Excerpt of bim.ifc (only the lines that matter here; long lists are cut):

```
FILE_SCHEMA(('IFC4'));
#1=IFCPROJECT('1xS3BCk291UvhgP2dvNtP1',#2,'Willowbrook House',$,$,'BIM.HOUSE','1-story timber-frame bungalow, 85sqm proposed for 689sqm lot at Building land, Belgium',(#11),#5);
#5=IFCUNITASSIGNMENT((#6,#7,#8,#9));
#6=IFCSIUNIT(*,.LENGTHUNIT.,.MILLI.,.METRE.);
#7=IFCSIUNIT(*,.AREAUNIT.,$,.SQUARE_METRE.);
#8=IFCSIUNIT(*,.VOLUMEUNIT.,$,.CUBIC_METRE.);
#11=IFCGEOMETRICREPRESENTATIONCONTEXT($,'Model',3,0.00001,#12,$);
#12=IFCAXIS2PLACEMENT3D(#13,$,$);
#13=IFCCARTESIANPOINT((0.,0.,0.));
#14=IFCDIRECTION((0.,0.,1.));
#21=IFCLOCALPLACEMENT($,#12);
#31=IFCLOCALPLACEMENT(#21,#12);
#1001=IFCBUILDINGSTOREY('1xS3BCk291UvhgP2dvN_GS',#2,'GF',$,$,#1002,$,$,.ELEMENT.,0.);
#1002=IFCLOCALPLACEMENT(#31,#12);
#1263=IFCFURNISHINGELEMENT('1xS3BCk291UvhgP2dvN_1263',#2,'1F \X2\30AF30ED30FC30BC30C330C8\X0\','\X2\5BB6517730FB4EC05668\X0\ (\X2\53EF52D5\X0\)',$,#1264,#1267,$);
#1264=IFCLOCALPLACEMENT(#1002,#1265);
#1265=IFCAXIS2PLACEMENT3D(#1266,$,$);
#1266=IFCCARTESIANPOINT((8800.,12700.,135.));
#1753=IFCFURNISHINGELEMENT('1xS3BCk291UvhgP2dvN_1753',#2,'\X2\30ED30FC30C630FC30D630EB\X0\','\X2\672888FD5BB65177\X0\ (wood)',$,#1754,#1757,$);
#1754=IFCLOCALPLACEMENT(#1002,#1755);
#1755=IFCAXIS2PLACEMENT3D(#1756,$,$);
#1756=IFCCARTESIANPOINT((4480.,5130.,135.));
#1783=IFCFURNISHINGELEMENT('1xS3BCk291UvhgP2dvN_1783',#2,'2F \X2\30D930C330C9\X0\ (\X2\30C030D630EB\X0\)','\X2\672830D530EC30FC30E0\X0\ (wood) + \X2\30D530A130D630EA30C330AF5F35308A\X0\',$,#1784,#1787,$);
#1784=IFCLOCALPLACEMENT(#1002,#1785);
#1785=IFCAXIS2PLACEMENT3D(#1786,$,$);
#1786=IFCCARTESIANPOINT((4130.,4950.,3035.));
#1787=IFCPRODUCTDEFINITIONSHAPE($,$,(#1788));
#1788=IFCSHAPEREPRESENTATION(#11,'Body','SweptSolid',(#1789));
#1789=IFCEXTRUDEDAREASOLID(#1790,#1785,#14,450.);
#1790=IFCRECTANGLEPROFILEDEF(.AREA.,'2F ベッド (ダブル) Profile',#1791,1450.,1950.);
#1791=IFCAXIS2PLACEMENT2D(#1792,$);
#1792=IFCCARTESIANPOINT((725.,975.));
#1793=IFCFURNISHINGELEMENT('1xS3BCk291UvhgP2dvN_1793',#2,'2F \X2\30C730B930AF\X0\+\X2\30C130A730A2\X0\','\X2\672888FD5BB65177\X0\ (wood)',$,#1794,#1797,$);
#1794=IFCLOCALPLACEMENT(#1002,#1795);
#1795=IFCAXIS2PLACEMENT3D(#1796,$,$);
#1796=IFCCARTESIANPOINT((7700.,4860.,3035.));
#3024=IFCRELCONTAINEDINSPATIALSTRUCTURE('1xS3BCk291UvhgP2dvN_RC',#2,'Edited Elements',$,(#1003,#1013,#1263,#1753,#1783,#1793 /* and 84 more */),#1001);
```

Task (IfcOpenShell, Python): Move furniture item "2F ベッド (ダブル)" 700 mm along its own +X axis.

```python
import ifcopenshell
import ifcopenshell.api.geometry
import ifcopenshell.util.placement
import ifcopenshell.util.unit

model = ifcopenshell.open("bim.ifc")
unit_scale = ifcopenshell.util.unit.calculate_unit_scale(model)

item = model.by_guid("1xS3BCk291UvhgP2dvN_1783")
matrix = ifcopenshell.util.placement.get_local_placement(item.ObjectPlacement)
matrix[:3, 3] += matrix[:3, 0] * 0.7 / unit_scale
ifcopenshell.api.geometry.edit_object_placement(model, product=item, matrix=matrix, is_si=False)

print(ifcopenshell.util.placement.get_local_placement(item.ObjectPlacement).round(3) + 0.0)

model.write("bim-out.ifc")
```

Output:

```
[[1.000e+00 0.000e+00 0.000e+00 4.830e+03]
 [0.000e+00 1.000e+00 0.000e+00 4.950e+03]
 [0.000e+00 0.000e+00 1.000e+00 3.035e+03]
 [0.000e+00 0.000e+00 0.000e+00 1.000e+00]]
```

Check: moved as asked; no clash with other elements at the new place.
